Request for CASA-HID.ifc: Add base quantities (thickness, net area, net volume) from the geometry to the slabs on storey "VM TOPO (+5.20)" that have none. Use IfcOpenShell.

First a look at what the model holds.

```python
import ifcopenshell
import ifcopenshell.util.element
import ifcopenshell.util.unit

model = ifcopenshell.open("CASA-HID.ifc")
print(model.schema)
for unit_type in ("LENGTHUNIT", "AREAUNIT", "VOLUMEUNIT"):
    print(unit_type, ifcopenshell.util.unit.calculate_unit_scale(model, unit_type))
storey = next(s for s in model.by_type("IfcBuildingStorey") if s.Name == "VM TOPO (+5.20)")
slabs = [e for e in ifcopenshell.util.element.get_decomposition(storey) if e.is_a("IfcSlab")]
for e in sorted(slabs, key=lambda e: e.id()):
    print(e.id(), e.is_a(), e.Name, list(ifcopenshell.util.element.get_psets(e, qtos_only=True)), sep=" | ")
```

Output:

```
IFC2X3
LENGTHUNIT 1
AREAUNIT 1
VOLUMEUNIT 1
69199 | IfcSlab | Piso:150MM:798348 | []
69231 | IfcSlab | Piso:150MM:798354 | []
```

```python
import ifcopenshell
import ifcopenshell.api.pset
import ifcopenshell.geom
import ifcopenshell.util.element
import ifcopenshell.util.shape
import ifcopenshell.util.unit

model = ifcopenshell.open("CASA-HID.ifc")
unit_scale = ifcopenshell.util.unit.calculate_unit_scale(model)
area_scale = ifcopenshell.util.unit.calculate_unit_scale(model, "AREAUNIT")
volume_scale = ifcopenshell.util.unit.calculate_unit_scale(model, "VOLUMEUNIT")
settings = ifcopenshell.geom.settings()

storey = next(s for s in model.by_type("IfcBuildingStorey") if s.Name == "VM TOPO (+5.20)")
slabs = [e for e in ifcopenshell.util.element.get_decomposition(storey) if e.is_a("IfcSlab")]

for e in sorted(slabs, key=lambda e: e.id()):
    if ifcopenshell.util.element.get_psets(e, qtos_only=True, should_inherit=False):
        continue
    # Geometry comes back in metres, in the element's own axes.
    shape = ifcopenshell.geom.create_shape(settings, e)
    values = {
        "Width": ifcopenshell.util.shape.get_z(shape.geometry) / unit_scale,
        "NetArea": ifcopenshell.util.shape.get_footprint_area(shape.geometry) / area_scale,
        "NetVolume": ifcopenshell.util.shape.get_volume(shape.geometry) / volume_scale,
    }
    qto = ifcopenshell.api.pset.add_qto(model, product=e, name="BaseQuantities")
    ifcopenshell.api.pset.edit_qto(model, qto=qto, properties=values)
    print(e.id(), {k: round(v, 3) for k, v in values.items()})

model.write("CASA-HID-out.ifc")
```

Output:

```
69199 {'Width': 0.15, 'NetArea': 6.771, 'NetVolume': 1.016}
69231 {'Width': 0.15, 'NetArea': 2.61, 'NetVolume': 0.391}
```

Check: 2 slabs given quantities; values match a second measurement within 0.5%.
